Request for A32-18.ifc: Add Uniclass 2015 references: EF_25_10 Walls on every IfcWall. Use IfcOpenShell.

First a look at what the model holds.

```python
import ifcopenshell

model = ifcopenshell.open("A32-18.ifc")
print(model.schema)
print("classifications:", [c.Name for c in model.by_type("IfcClassification")])
for ifc_class in ("IfcDoor", "IfcRoof", "IfcStair", "IfcWall", "IfcWindow"):
    print(ifc_class, len(model.by_type(ifc_class)))
```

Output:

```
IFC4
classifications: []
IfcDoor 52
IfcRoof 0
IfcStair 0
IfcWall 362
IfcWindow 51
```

```python
import ifcopenshell
import ifcopenshell.api.classification

model = ifcopenshell.open("A32-18.ifc")

system = ifcopenshell.api.classification.add_classification(model, classification="Uniclass 2015")

codes = {
    "IfcWall": ("EF_25_10", "Walls"),
}
for ifc_class, (code, name) in codes.items():
    products = model.by_type(ifc_class)
    ifcopenshell.api.classification.add_reference(
        model, products=products, classification=system, identification=code, name=name
    )
    print(code, len(products))

model.write("A32-18-out.ifc")
```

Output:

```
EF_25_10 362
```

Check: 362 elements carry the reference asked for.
